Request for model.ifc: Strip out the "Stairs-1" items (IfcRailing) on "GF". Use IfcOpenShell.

First a look at what the model holds.

```python
import ifcopenshell
import ifcopenshell.util.element

model = ifcopenshell.open("model.ifc")
print(model.schema)
storey = next(s for s in model.by_type("IfcBuildingStorey") if s.Name == "GF")
railings = [e for e in ifcopenshell.util.element.get_decomposition(storey) if e.is_a("IfcRailing")]
seen = {}
for e in railings:
    element_type = ifcopenshell.util.element.get_type(e)
    name = element_type.Name if element_type not in (None, e) else None
    seen[name] = seen.get(name, 0) + 1
for name, count in sorted(seen.items(), key=str):
    print(count, "x", name)
```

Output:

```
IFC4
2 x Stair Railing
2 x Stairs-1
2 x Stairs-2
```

```python
import ifcopenshell
import ifcopenshell.api.root
import ifcopenshell.util.element

model = ifcopenshell.open("model.ifc")

storey = next(s for s in model.by_type("IfcBuildingStorey") if s.Name == "GF")
railings = [e for e in ifcopenshell.util.element.get_decomposition(storey) if e.is_a("IfcRailing")]
targets = [e for e in railings if (t := ifcopenshell.util.element.get_type(e)) not in (None, e) and t.Name == "Stairs-1"]

for e in targets:
    ifcopenshell.api.root.remove_product(model, product=e)
print(len(targets), "removed")

model.write("model-out.ifc")
```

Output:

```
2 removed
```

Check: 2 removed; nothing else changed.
